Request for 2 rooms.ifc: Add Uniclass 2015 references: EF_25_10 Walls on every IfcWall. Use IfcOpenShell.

First a look at what the model holds.

```python
import ifcopenshell

model = ifcopenshell.open("2 rooms.ifc")
print(model.schema)
print("classifications:", [c.Name for c in model.by_type("IfcClassification")])
for ifc_class in ("IfcDoor", "IfcRoof", "IfcStair", "IfcWall", "IfcWindow"):
    print(ifc_class, len(model.by_type(ifc_class)))
```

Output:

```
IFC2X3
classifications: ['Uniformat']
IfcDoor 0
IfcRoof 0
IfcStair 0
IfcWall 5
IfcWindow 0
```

```python
import ifcopenshell
import ifcopenshell.api.classification

model = ifcopenshell.open("2 rooms.ifc")

# IFC2X3 requires Source and Edition and has no link from the project to the system.
system = model.create_entity("IfcClassification", Source="NBS", Edition="2015", Name="Uniclass 2015")

codes = {
    "IfcWall": ("EF_25_10", "Walls"),
}
for ifc_class, (code, name) in codes.items():
    products = model.by_type(ifc_class)
    ifcopenshell.api.classification.add_reference(
        model, products=products, classification=system, identification=code, name=name
    )
    print(code, len(products))

model.write("2 rooms_updated.ifc")
```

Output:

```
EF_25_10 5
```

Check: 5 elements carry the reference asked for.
